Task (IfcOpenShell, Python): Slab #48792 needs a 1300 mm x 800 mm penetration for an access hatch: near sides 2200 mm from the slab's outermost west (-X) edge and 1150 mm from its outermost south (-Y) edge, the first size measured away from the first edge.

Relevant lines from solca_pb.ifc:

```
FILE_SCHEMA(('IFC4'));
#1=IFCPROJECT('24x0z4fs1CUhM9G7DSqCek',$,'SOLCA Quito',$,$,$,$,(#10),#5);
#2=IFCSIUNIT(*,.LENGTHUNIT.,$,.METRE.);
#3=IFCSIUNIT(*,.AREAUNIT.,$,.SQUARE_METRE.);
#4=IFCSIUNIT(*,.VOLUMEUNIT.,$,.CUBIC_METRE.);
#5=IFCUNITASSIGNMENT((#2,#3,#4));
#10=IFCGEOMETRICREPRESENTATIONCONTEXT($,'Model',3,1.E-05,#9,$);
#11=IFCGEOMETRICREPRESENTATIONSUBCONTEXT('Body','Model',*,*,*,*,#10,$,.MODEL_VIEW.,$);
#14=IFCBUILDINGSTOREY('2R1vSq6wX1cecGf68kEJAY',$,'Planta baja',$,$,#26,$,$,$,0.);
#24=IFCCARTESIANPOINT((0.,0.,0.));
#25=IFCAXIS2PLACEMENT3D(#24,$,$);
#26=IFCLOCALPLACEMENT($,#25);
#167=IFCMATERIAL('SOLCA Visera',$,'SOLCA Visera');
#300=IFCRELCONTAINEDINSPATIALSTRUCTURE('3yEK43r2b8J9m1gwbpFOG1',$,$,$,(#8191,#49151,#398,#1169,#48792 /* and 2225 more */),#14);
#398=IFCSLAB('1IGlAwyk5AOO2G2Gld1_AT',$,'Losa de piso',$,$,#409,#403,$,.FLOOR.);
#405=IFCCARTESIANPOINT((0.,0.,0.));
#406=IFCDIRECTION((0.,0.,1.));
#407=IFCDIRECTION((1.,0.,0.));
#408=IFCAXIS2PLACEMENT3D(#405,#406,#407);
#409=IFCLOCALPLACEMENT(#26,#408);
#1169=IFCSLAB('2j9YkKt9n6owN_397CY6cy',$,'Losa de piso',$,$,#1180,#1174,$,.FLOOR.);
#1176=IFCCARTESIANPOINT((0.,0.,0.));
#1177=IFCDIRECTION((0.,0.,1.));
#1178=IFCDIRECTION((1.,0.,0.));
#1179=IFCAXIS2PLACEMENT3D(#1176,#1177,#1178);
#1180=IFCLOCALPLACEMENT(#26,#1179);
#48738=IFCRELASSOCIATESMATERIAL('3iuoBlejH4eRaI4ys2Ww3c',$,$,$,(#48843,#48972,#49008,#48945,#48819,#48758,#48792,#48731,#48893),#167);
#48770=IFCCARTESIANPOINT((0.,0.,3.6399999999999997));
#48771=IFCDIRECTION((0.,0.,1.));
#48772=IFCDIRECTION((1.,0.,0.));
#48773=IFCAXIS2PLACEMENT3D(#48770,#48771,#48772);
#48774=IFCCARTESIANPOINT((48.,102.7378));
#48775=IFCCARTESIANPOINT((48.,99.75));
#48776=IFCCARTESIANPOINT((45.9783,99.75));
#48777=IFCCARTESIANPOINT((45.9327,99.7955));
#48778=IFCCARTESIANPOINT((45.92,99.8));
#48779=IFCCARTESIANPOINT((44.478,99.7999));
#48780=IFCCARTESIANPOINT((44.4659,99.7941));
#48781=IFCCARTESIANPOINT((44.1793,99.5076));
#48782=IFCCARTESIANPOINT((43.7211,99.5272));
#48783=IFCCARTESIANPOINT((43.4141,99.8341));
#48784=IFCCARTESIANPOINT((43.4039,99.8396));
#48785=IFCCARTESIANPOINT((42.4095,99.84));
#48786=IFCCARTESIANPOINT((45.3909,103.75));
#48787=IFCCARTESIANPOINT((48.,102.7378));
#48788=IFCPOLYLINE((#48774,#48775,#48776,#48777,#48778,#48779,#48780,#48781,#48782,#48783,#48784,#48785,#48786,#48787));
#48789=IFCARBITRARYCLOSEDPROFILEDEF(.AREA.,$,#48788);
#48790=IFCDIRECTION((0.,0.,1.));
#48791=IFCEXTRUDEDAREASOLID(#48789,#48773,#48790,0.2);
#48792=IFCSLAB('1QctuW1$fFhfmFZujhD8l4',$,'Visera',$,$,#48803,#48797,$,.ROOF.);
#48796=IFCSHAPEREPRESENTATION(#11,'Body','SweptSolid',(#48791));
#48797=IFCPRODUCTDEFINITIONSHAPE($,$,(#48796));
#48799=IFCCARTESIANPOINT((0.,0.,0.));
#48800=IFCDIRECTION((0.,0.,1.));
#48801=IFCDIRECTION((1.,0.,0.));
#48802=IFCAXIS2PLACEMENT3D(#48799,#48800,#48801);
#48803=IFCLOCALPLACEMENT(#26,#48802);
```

```python
import numpy as np
import ifcopenshell
import ifcopenshell.api.feature
import ifcopenshell.api.geometry
import ifcopenshell.api.root
import ifcopenshell.geom
import ifcopenshell.util.placement
import ifcopenshell.util.representation
import ifcopenshell.util.shape
import ifcopenshell.util.unit

model = ifcopenshell.open("solca_pb.ifc")
unit_scale = ifcopenshell.util.unit.calculate_unit_scale(model)
settings = ifcopenshell.geom.settings()


def volume(element):
    """Net volume in cubic metres, openings subtracted."""
    shape = ifcopenshell.geom.create_shape(settings, element)
    return ifcopenshell.util.shape.get_volume(shape.geometry)


slab = model.by_guid("1QctuW1$fFhfmFZujhD8l4")
before = volume(slab)

# Extent in the slab's own axes, in metres. The edges named are its -X and -Y sides.
slab_shape = ifcopenshell.geom.create_shape(settings, slab)
vertices = ifcopenshell.util.shape.get_vertices(slab_shape.geometry)
x_min, y_min, bottom = vertices.min(axis=0)
top = vertices[:, 2].max()

opening = ifcopenshell.api.root.create_entity(model, ifc_class="IfcOpeningElement", name="Access hatch opening", predefined_type="OPENING")
context = ifcopenshell.util.representation.get_context(model, "Model", "Body", "MODEL_VIEW")
width, depth = 1.3, 0.8
outline = [(0.0, 0.0), (width, 0.0), (width, depth), (0.0, depth), (0.0, 0.0)]
# Overshoot both faces by 50 mm so the cut is clean.
shape = ifcopenshell.api.geometry.add_slab_representation(
    model, context=context, depth=top - bottom + 0.1, polyline=outline
)
ifcopenshell.api.geometry.assign_representation(model, product=opening, representation=shape)

matrix = ifcopenshell.util.placement.get_local_placement(slab.ObjectPlacement)
matrix[:, 3] = matrix @ np.append(np.array([x_min + 2.2, y_min + 1.15, bottom - 0.05]) / unit_scale, 1.0)
ifcopenshell.api.geometry.edit_object_placement(model, product=opening, matrix=matrix, is_si=False)
ifcopenshell.api.feature.add_feature(model, feature=opening, element=slab)

after = volume(slab)

print(f"slab volume {before:.3f} -> {after:.3f} m3")

model.write("solca_pb-out.ifc")
```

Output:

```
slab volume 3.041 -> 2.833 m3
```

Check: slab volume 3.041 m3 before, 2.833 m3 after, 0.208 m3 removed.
